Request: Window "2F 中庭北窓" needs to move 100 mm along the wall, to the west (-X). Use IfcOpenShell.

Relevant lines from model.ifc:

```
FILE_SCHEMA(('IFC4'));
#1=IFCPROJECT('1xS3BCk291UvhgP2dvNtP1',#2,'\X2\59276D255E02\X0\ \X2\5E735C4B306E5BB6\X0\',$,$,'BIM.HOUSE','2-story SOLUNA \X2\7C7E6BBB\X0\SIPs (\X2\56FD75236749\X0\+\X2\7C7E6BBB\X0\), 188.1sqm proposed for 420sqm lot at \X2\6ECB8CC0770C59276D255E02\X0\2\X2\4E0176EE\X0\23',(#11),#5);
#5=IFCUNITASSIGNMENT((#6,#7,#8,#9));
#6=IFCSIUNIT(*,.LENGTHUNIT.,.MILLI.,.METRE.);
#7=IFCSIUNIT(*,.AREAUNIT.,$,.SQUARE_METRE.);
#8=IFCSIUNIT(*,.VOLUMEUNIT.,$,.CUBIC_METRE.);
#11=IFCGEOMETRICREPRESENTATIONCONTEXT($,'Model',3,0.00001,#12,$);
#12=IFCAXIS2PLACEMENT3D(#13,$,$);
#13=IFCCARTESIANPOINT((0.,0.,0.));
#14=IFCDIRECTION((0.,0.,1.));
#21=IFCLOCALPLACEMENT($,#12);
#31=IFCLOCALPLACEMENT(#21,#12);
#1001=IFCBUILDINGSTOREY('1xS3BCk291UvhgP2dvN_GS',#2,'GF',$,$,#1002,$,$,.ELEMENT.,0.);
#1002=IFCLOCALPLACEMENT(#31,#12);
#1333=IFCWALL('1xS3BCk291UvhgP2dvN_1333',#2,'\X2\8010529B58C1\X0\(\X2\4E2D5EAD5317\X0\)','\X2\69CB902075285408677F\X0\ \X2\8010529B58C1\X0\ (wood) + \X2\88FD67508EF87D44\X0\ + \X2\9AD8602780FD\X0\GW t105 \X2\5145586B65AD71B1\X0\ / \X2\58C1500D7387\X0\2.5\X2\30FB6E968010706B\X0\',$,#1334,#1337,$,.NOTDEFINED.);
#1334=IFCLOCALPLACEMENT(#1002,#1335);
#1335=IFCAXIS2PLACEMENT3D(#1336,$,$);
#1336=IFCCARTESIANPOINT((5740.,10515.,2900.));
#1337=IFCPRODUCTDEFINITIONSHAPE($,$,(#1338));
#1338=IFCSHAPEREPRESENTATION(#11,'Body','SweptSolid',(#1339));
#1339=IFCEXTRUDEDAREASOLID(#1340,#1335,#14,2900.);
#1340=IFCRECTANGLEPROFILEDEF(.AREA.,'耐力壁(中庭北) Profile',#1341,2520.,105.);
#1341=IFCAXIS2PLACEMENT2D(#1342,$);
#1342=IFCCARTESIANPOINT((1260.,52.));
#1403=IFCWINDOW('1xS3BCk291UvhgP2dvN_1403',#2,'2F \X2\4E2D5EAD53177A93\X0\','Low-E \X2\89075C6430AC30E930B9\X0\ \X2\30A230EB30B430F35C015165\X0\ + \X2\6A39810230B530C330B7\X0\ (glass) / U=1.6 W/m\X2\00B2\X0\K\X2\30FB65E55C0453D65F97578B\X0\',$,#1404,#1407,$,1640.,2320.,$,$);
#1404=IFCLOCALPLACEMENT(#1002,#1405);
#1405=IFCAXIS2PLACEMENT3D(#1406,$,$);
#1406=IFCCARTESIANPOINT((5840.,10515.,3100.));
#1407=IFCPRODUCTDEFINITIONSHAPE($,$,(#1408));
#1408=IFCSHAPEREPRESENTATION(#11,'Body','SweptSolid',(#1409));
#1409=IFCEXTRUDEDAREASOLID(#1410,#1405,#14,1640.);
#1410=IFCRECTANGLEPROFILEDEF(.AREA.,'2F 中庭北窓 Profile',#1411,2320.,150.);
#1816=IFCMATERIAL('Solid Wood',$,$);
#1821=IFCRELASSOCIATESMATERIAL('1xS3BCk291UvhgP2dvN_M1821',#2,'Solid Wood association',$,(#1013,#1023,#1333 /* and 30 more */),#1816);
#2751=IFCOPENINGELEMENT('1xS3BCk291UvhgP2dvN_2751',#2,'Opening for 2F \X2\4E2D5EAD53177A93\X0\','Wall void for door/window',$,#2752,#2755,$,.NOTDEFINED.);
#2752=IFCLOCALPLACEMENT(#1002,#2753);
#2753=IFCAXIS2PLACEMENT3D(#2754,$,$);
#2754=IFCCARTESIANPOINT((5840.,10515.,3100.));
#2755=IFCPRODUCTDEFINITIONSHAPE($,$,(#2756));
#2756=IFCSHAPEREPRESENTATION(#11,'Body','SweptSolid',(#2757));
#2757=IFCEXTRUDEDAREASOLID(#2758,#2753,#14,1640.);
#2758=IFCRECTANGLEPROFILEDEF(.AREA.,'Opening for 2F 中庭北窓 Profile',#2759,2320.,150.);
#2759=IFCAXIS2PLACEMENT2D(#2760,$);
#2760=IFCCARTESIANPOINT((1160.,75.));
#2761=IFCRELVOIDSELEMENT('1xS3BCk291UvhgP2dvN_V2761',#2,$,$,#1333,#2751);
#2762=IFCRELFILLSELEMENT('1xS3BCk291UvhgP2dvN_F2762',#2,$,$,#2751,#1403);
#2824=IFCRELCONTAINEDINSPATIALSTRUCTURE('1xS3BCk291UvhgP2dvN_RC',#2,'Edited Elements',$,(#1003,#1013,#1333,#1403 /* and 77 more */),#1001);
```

```python
import ifcopenshell
import ifcopenshell.api.geometry
import ifcopenshell.util.placement
import ifcopenshell.util.unit

model = ifcopenshell.open("model.ifc")
unit_scale = ifcopenshell.util.unit.calculate_unit_scale(model)

window = model.by_guid("1xS3BCk291UvhgP2dvN_1403")
opening = window.FillsVoids[0].RelatingOpeningElement
wall = opening.VoidsElements[0].RelatingBuildingElement

wall_matrix = ifcopenshell.util.placement.get_local_placement(wall.ObjectPlacement)
shift = wall_matrix[:3, 0] * -0.1 / unit_scale
before = ifcopenshell.util.placement.get_local_placement(window.ObjectPlacement)[:3, 3].copy()

# The window is not placed relative to its opening, so move both.
for product in (opening, window):
    matrix = ifcopenshell.util.placement.get_local_placement(product.ObjectPlacement)
    matrix[:3, 3] += shift
    ifcopenshell.api.geometry.edit_object_placement(model, product=product, matrix=matrix, is_si=False)

after = ifcopenshell.util.placement.get_local_placement(window.ObjectPlacement)[:3, 3]
print("window moved by", (after - before).round(3) + 0.0)

model.write("model_v2.ifc")
```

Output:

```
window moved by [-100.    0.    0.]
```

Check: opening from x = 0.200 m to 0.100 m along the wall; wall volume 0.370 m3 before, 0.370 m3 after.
